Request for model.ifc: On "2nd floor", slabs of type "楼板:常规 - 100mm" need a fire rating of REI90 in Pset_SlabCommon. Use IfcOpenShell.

First a look at what the model holds.

```python
import ifcopenshell
import ifcopenshell.util.element

model = ifcopenshell.open("model.ifc")
print(model.schema)
storey = next(s for s in model.by_type("IfcBuildingStorey") if s.Name == "2nd floor")
slabs = [e for e in ifcopenshell.util.element.get_decomposition(storey) if e.is_a("IfcSlab")]
seen = {}
for e in slabs:
    element_type = ifcopenshell.util.element.get_type(e)
    key = (element_type.Name if element_type != e and element_type else None, ifcopenshell.util.element.get_pset(e, "Pset_SlabCommon", "FireRating"))
    seen[key] = seen.get(key, 0) + 1
for (name, value), count in sorted(seen.items(), key=str):
    print(count, "x", name, "|", value)
```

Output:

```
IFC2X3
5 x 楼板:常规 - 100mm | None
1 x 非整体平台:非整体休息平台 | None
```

```python
import ifcopenshell
import ifcopenshell.api.pset
import ifcopenshell.util.element

model = ifcopenshell.open("model.ifc")

storey = next(s for s in model.by_type("IfcBuildingStorey") if s.Name == "2nd floor")
slabs = [e for e in ifcopenshell.util.element.get_decomposition(storey) if e.is_a("IfcSlab")]

count = 0
for e in slabs:
    element_type = ifcopenshell.util.element.get_type(e)
    if element_type in (None, e) or element_type.Name != "楼板:常规 - 100mm":
        continue
    # add_pset returns the element's existing set when there is one.
    pset = ifcopenshell.api.pset.add_pset(model, product=e, name="Pset_SlabCommon")
    ifcopenshell.api.pset.edit_pset(model, pset=pset, properties={"FireRating": "REI90"})
    count += 1

print(count, "slabs updated")

model.write("model_edited.ifc")
```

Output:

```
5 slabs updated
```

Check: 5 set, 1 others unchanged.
